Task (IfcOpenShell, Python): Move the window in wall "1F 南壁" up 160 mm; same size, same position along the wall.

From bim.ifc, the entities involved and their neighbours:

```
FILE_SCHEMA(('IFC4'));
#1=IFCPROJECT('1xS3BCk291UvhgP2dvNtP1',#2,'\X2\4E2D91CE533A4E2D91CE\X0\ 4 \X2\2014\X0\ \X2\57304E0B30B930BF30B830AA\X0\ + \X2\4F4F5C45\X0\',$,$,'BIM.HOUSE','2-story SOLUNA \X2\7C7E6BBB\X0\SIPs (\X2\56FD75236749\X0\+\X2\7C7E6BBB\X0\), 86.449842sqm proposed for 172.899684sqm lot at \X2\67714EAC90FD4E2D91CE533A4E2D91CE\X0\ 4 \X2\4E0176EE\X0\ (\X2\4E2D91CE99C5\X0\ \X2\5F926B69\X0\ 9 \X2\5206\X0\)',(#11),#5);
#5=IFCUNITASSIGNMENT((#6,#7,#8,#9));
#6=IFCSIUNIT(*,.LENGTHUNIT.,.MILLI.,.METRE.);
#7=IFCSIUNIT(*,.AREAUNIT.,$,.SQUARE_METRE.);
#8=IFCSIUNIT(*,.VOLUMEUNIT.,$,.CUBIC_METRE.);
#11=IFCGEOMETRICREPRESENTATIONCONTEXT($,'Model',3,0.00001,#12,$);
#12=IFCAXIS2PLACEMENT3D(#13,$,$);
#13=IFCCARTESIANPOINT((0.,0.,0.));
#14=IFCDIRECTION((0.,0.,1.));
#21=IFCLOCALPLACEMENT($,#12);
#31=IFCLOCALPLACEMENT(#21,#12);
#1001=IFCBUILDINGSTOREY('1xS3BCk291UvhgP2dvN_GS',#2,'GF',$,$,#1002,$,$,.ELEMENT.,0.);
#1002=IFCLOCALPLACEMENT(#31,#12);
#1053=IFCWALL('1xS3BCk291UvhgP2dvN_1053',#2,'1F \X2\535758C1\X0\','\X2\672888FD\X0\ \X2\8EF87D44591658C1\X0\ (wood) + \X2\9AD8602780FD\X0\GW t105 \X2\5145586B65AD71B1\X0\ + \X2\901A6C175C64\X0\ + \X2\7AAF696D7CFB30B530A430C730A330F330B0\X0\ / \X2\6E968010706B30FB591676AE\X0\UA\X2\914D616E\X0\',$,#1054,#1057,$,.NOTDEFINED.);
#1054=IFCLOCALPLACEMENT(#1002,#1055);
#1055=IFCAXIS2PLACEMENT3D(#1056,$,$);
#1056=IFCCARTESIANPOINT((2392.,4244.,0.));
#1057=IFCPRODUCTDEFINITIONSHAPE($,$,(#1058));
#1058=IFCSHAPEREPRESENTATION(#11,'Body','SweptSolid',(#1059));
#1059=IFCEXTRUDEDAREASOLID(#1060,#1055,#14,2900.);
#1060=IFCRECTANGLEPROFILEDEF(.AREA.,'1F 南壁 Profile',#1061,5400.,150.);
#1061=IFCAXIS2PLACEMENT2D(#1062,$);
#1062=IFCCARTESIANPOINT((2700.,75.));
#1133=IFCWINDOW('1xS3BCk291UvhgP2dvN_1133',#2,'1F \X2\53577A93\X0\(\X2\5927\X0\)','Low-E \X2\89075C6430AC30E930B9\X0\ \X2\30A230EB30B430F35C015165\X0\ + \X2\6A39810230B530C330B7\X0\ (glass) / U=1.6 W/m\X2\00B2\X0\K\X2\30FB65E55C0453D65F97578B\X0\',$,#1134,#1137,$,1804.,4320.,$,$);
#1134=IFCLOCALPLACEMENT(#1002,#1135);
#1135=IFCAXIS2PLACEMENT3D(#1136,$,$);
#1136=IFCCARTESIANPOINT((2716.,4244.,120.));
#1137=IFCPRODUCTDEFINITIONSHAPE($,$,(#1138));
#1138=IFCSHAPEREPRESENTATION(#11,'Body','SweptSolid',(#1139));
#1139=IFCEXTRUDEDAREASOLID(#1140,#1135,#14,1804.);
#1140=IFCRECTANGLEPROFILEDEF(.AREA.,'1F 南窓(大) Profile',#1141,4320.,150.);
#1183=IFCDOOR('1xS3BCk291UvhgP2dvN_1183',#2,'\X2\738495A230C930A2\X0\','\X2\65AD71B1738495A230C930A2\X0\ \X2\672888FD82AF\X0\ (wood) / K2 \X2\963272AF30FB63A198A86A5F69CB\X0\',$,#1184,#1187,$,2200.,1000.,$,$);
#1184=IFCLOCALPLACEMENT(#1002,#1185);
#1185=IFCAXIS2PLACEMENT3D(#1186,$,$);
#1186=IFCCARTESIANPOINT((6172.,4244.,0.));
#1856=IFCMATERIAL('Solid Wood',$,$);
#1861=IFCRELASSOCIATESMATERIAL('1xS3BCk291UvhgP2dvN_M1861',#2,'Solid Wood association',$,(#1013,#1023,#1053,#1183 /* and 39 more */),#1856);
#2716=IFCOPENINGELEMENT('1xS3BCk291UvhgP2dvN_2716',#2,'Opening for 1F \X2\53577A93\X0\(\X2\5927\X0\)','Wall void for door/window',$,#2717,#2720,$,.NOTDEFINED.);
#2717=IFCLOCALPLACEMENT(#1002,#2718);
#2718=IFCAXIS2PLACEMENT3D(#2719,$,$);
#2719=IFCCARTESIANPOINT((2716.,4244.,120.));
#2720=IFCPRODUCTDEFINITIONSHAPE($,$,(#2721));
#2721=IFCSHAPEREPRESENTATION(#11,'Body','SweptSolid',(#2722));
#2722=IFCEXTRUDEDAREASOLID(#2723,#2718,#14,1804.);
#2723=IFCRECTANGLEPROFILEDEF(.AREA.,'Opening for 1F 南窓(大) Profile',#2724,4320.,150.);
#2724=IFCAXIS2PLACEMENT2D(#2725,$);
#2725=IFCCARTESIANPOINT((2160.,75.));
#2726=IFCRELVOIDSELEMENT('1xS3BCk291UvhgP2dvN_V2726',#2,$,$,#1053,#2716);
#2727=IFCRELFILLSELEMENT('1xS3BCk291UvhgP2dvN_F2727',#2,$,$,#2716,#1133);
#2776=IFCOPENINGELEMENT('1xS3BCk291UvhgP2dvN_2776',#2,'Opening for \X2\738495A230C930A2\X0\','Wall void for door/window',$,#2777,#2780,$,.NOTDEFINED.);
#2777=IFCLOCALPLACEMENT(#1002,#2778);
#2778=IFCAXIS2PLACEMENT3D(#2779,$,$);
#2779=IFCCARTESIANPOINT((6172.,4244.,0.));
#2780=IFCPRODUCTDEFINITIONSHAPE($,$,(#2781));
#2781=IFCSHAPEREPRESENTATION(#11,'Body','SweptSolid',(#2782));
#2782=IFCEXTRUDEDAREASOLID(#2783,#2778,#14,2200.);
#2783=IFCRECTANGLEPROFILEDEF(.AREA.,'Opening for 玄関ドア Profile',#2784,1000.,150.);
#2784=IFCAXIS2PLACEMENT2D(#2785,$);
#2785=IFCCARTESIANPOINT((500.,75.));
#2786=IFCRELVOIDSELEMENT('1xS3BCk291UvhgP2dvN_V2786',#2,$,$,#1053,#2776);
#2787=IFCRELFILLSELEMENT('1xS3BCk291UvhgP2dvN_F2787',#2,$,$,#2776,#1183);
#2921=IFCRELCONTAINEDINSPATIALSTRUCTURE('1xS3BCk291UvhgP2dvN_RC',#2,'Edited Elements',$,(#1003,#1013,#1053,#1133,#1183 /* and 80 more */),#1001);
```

```python
import numpy as np
import ifcopenshell
import ifcopenshell.api.geometry
import ifcopenshell.util.placement
import ifcopenshell.util.unit

model = ifcopenshell.open("bim.ifc")
unit_scale = ifcopenshell.util.unit.calculate_unit_scale(model)

window = model.by_id(1133)
opening = window.FillsVoids[0].RelatingOpeningElement
dz = 0.16 / unit_scale

shift = np.array([0.0, 0.0, dz])
# The window is not placed relative to its opening, so move both.
for product in (opening, window):
    matrix = ifcopenshell.util.placement.get_local_placement(product.ObjectPlacement)
    matrix[:3, 3] += shift
    ifcopenshell.api.geometry.edit_object_placement(model, product=product, matrix=matrix, is_si=False)

print(f"moved by {dz * unit_scale:+.3f} m")

model.write("bim_edited.ifc")
```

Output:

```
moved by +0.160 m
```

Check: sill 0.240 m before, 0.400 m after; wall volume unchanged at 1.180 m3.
